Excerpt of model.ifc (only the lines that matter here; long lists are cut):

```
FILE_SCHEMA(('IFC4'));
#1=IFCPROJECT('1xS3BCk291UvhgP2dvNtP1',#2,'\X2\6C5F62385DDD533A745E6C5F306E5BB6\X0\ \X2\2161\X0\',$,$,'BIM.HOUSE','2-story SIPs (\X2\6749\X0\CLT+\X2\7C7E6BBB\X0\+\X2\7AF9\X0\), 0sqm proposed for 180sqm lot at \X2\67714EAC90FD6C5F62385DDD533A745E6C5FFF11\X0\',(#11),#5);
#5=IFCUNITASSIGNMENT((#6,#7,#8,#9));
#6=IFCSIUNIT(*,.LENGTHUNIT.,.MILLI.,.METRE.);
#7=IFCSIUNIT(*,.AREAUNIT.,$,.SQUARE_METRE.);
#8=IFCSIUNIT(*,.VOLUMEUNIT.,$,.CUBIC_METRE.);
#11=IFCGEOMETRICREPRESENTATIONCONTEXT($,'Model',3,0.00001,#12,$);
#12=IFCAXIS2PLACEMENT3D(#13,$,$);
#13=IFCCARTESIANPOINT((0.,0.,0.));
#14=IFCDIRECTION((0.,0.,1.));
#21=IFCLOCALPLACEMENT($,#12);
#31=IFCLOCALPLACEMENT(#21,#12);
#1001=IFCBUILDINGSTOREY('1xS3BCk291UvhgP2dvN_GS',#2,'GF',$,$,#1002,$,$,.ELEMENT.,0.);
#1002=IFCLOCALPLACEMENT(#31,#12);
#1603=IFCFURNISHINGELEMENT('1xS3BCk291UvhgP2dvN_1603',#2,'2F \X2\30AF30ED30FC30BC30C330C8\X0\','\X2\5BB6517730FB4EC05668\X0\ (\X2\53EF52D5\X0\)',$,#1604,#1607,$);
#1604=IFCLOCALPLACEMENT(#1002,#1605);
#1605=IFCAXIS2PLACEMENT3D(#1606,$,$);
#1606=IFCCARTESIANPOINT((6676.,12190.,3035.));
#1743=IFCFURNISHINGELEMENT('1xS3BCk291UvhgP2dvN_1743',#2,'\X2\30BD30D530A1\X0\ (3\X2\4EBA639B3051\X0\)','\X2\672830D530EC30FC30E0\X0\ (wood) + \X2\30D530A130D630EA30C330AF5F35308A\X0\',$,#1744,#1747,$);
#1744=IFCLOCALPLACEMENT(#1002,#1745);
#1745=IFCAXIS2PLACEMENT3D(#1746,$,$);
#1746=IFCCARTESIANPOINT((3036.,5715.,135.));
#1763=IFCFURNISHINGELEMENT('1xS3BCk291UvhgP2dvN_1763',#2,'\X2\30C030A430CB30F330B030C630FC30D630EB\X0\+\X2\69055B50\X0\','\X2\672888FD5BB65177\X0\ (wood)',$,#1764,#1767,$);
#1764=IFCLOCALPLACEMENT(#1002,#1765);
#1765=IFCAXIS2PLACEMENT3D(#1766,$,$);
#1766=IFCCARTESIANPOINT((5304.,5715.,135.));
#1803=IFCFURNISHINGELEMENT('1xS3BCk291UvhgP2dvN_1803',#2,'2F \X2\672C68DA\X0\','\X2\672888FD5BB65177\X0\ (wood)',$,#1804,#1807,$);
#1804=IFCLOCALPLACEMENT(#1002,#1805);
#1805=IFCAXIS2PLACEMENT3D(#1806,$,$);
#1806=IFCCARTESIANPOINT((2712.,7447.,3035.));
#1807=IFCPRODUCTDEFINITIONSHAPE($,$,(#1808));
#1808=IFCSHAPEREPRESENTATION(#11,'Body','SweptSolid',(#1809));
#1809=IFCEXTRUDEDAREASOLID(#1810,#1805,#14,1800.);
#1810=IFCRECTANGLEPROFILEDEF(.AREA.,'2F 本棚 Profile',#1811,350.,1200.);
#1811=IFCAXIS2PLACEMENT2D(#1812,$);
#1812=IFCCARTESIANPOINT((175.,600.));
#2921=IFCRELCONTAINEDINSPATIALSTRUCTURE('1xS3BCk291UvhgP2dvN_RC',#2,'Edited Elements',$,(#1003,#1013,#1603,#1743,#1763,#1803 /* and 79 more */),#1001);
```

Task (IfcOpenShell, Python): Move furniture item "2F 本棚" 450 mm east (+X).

```python
import ifcopenshell
import ifcopenshell.api.geometry
import ifcopenshell.util.placement
import ifcopenshell.util.unit

model = ifcopenshell.open("model.ifc")
unit_scale = ifcopenshell.util.unit.calculate_unit_scale(model)

item = model.by_guid("1xS3BCk291UvhgP2dvN_1803")
matrix = ifcopenshell.util.placement.get_local_placement(item.ObjectPlacement)
matrix[0, 3] += 0.45 / unit_scale
ifcopenshell.api.geometry.edit_object_placement(model, product=item, matrix=matrix, is_si=False)

print(ifcopenshell.util.placement.get_local_placement(item.ObjectPlacement).round(3) + 0.0)

model.write("model_rev.ifc")
```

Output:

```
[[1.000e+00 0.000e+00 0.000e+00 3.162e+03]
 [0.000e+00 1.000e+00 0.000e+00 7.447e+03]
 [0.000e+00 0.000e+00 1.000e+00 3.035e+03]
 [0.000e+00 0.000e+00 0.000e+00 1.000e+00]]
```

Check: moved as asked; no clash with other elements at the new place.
